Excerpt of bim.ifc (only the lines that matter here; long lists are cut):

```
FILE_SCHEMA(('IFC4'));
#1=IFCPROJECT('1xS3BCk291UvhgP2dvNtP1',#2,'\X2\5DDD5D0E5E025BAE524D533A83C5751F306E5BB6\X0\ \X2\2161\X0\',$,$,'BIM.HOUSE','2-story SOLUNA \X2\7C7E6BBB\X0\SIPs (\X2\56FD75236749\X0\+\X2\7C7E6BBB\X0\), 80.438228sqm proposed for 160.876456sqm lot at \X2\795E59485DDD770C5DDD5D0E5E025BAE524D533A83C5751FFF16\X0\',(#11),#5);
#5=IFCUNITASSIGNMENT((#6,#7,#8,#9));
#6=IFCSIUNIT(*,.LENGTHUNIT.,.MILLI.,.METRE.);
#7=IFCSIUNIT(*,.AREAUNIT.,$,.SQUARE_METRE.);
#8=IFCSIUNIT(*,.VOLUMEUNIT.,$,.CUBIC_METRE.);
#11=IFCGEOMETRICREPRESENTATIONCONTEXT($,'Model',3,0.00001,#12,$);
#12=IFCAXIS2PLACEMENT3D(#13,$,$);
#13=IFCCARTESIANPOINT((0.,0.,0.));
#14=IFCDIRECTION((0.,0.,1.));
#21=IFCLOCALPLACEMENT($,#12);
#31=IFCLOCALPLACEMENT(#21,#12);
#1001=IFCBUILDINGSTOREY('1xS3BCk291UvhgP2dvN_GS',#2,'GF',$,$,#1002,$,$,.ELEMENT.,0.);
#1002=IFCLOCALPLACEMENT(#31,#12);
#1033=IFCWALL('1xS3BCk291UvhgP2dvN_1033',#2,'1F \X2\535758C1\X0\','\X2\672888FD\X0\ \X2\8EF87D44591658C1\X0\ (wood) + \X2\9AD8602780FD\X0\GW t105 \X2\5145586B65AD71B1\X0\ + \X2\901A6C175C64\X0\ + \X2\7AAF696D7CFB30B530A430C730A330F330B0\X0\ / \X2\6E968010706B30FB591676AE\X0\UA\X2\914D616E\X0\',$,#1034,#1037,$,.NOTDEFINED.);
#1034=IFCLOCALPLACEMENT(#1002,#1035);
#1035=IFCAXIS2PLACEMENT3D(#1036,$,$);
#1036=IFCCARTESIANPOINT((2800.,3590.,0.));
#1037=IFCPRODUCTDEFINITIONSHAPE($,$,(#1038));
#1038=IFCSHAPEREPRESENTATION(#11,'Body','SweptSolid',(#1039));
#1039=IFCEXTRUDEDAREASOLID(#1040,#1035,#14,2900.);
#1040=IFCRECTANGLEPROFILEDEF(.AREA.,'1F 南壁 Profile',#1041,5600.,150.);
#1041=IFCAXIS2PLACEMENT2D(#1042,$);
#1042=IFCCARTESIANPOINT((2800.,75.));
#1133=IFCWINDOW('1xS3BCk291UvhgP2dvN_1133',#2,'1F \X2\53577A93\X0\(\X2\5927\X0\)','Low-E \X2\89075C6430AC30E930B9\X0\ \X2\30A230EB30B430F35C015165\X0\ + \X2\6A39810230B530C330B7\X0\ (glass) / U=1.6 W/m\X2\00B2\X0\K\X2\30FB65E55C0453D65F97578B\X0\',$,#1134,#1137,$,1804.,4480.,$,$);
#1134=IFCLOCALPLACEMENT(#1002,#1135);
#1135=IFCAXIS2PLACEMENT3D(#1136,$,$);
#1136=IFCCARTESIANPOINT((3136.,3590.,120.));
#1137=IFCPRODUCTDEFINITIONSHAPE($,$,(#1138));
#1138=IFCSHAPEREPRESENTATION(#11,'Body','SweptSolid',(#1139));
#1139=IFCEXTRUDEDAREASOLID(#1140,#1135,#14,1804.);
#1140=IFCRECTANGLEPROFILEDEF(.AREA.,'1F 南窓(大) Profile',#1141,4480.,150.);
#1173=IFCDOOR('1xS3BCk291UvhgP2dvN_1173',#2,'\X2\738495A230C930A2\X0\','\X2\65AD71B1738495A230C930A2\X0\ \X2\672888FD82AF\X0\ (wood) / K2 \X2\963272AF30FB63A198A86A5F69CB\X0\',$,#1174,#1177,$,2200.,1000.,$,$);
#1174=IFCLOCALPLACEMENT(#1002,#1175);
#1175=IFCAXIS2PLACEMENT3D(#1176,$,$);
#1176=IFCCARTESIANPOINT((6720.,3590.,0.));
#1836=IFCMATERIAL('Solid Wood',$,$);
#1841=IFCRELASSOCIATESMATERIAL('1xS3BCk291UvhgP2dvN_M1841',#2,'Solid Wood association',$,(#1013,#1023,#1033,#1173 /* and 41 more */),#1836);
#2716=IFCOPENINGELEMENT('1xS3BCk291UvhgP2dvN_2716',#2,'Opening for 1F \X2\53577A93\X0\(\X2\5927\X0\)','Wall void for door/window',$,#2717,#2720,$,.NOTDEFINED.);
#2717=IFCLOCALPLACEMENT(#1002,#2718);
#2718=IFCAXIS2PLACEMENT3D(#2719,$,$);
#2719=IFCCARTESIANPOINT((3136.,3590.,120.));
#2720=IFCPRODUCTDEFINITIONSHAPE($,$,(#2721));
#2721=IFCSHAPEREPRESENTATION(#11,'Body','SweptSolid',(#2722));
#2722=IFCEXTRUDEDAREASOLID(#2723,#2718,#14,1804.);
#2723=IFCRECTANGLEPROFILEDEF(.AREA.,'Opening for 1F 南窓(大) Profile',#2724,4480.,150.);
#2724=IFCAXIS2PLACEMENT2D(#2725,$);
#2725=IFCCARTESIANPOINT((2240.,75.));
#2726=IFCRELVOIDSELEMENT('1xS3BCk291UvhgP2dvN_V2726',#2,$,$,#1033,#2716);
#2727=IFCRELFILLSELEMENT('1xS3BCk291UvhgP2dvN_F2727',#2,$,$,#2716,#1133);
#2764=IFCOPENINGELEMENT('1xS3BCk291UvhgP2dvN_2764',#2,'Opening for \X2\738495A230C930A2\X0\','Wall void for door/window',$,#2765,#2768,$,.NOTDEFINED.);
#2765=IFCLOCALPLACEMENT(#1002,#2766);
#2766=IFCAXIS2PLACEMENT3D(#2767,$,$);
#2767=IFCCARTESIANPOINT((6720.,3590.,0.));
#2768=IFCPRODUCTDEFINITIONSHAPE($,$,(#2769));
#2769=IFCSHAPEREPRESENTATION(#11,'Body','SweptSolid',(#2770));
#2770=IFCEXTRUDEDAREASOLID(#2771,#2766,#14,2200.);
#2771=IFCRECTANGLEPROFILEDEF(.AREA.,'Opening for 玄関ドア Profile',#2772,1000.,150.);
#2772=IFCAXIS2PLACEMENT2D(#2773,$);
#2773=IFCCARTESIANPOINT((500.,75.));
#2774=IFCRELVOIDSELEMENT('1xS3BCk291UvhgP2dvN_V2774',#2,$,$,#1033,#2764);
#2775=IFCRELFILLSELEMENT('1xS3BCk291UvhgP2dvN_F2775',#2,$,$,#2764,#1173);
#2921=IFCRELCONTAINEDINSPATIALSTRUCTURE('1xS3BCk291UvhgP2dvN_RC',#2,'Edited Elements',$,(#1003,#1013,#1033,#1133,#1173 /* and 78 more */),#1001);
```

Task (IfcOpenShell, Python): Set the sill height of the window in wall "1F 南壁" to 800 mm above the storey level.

```python
import numpy as np
import ifcopenshell
import ifcopenshell.api.geometry
import ifcopenshell.geom
import ifcopenshell.util.element
import ifcopenshell.util.placement
import ifcopenshell.util.shape
import ifcopenshell.util.unit

model = ifcopenshell.open("bim.ifc")
unit_scale = ifcopenshell.util.unit.calculate_unit_scale(model)

window = model.by_id(1133)
opening = window.FillsVoids[0].RelatingOpeningElement
storey = ifcopenshell.util.element.get_container(window, ifc_class="IfcBuildingStorey")
level = ifcopenshell.util.placement.get_local_placement(storey.ObjectPlacement)[2, 3]

# The opening's origin need not be at the sill, so measure its lowest point.
shape = ifcopenshell.geom.create_shape(ifcopenshell.geom.settings(), opening)
bottom = ifcopenshell.util.shape.get_shape_bottom_elevation(shape, shape.geometry) / unit_scale
dz = level + 800.0 - bottom

shift = np.array([0.0, 0.0, dz])
# The window is not placed relative to its opening, so move both.
for product in (opening, window):
    matrix = ifcopenshell.util.placement.get_local_placement(product.ObjectPlacement)
    matrix[:3, 3] += shift
    ifcopenshell.api.geometry.edit_object_placement(model, product=product, matrix=matrix, is_si=False)

print(f"moved by {dz * unit_scale:+.3f} m")

model.write("bim_updated.ifc")
```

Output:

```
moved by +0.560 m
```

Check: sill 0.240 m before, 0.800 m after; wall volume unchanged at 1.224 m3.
